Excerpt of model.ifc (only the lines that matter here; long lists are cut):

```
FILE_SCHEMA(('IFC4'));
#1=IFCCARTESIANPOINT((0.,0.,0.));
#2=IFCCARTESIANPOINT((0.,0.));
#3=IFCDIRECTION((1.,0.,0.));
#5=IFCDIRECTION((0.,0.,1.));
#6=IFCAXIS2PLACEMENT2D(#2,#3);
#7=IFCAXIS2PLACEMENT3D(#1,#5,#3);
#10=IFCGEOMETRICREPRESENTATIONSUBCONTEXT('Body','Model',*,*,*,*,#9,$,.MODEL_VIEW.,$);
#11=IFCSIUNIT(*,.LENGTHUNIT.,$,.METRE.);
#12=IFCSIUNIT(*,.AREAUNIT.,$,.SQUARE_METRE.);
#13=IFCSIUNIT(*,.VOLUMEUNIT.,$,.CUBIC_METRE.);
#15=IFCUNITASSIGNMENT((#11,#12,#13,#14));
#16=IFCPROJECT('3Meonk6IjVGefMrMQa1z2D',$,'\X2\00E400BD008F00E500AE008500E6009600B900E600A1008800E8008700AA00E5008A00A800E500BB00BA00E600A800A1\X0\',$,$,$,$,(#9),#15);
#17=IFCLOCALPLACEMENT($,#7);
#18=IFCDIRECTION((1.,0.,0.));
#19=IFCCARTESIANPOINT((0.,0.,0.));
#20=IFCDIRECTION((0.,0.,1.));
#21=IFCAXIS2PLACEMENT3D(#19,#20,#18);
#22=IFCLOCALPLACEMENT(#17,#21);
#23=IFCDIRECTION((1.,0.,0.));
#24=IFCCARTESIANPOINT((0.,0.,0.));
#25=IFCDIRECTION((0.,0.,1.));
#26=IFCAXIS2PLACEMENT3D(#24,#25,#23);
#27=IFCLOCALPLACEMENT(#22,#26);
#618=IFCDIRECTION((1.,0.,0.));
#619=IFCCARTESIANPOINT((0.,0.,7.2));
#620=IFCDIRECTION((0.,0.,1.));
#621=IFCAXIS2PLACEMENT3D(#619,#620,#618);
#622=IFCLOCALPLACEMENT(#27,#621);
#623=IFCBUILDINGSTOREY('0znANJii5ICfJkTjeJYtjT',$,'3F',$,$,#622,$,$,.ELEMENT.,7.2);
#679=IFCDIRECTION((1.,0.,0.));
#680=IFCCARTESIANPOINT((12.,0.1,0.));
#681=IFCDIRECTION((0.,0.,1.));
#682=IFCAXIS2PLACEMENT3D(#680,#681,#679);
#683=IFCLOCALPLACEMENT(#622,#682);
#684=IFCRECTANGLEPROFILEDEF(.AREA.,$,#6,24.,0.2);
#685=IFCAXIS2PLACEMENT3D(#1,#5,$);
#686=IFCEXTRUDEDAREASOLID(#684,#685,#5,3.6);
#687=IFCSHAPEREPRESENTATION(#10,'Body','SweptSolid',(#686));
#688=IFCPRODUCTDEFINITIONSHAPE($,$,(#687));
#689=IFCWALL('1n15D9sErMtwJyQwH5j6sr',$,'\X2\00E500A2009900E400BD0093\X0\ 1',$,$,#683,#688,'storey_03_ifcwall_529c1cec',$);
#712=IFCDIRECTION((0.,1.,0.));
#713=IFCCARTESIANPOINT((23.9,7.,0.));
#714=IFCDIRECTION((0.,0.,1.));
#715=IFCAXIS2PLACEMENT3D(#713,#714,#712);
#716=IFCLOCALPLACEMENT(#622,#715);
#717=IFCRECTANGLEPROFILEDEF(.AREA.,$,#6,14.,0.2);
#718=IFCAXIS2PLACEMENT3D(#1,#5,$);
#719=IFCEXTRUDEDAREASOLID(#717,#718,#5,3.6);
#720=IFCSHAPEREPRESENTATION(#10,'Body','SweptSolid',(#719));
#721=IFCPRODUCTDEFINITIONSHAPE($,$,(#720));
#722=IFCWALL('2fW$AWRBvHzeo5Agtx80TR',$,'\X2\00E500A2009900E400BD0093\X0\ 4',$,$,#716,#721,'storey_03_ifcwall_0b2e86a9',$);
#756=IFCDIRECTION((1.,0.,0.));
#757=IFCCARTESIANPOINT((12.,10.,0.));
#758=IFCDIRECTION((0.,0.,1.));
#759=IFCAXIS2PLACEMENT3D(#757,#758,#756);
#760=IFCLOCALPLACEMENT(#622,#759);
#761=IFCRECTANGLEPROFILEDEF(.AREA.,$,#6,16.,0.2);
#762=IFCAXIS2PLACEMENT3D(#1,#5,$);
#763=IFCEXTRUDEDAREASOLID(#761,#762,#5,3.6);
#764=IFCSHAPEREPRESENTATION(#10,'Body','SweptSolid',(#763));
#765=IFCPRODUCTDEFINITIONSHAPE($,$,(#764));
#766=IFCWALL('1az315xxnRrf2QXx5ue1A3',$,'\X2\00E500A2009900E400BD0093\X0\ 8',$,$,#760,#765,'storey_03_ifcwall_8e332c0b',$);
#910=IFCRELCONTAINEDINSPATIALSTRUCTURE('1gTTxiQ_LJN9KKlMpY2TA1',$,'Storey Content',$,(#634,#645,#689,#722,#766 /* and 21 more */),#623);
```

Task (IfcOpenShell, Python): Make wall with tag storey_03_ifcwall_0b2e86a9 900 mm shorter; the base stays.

```python
import ifcopenshell
import ifcopenshell.geom
import ifcopenshell.util.representation
import ifcopenshell.util.shape
import ifcopenshell.util.unit

model = ifcopenshell.open("model.ifc")
unit_scale = ifcopenshell.util.unit.calculate_unit_scale(model)
settings = ifcopenshell.geom.settings()


def volume(element):
    """Net volume in cubic metres, openings subtracted."""
    shape = ifcopenshell.geom.create_shape(settings, element)
    return ifcopenshell.util.shape.get_volume(shape.geometry)


wall = model.by_guid("2fW$AWRBvHzeo5Agtx80TR")
before = volume(wall)

body = ifcopenshell.util.representation.get_representation(wall, "Model", "Body")
solid = body.Items[0]
old_height = solid.Depth
solid.Depth -= 0.9 / unit_scale
after = volume(wall)

print(f"height {old_height:g} -> {solid.Depth:g}, volume {before:.3f} -> {after:.3f} m3")

model.write("model_updated.ifc")
```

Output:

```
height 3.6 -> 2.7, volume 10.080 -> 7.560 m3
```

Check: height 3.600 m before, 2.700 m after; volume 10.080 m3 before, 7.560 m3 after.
